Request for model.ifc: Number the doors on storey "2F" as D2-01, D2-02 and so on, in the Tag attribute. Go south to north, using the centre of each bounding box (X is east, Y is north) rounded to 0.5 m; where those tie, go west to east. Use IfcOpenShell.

First a look at what the model holds.

```python
import ifcopenshell
import ifcopenshell.util.element
import ifcopenshell.util.placement

model = ifcopenshell.open("model.ifc")
print(model.schema)
storey = next(s for s in model.by_type("IfcBuildingStorey") if s.Name == "2F")
doors = [e for e in ifcopenshell.util.element.get_decomposition(storey) if e.is_a("IfcDoor")]
for e in sorted(doors, key=lambda e: e.id()):
    origin = ifcopenshell.util.placement.get_local_placement(e.ObjectPlacement)[:3, 3]
    print(e.id(), e.Tag, e.Name, origin.round(2) + 0.0, sep=" | ")
```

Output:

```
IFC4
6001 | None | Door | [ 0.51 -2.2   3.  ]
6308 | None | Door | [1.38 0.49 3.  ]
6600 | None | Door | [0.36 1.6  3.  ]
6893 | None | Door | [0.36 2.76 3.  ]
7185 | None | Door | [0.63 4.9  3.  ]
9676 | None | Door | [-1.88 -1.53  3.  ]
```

```python
import ifcopenshell
import ifcopenshell.geom
import ifcopenshell.util.element
import ifcopenshell.util.shape

model = ifcopenshell.open("model.ifc")
settings = ifcopenshell.geom.settings()
settings.set("use-world-coords", True)


def centre(element):
    shape = ifcopenshell.geom.create_shape(settings, element)
    return ifcopenshell.util.shape.get_bbox_centroid(shape.geometry)


storey = next(s for s in model.by_type("IfcBuildingStorey") if s.Name == "2F")
doors = [e for e in ifcopenshell.util.element.get_decomposition(storey) if e.is_a("IfcDoor")]

# Insertion points can sit at a corner or the storey origin, so sort by the geometry (in metres).
centres = {e: centre(e) for e in doors}
doors.sort(key=lambda e: (round(centres[e][1] / 0.5), centres[e][0]))

for i, e in enumerate(doors, start=1):
    number = f"D2-{i:02d}"
    e.Tag = number
    print(e.id(), number)

model.write("model-out.ifc")
```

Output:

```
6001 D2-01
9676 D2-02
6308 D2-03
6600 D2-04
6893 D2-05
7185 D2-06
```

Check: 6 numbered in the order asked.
